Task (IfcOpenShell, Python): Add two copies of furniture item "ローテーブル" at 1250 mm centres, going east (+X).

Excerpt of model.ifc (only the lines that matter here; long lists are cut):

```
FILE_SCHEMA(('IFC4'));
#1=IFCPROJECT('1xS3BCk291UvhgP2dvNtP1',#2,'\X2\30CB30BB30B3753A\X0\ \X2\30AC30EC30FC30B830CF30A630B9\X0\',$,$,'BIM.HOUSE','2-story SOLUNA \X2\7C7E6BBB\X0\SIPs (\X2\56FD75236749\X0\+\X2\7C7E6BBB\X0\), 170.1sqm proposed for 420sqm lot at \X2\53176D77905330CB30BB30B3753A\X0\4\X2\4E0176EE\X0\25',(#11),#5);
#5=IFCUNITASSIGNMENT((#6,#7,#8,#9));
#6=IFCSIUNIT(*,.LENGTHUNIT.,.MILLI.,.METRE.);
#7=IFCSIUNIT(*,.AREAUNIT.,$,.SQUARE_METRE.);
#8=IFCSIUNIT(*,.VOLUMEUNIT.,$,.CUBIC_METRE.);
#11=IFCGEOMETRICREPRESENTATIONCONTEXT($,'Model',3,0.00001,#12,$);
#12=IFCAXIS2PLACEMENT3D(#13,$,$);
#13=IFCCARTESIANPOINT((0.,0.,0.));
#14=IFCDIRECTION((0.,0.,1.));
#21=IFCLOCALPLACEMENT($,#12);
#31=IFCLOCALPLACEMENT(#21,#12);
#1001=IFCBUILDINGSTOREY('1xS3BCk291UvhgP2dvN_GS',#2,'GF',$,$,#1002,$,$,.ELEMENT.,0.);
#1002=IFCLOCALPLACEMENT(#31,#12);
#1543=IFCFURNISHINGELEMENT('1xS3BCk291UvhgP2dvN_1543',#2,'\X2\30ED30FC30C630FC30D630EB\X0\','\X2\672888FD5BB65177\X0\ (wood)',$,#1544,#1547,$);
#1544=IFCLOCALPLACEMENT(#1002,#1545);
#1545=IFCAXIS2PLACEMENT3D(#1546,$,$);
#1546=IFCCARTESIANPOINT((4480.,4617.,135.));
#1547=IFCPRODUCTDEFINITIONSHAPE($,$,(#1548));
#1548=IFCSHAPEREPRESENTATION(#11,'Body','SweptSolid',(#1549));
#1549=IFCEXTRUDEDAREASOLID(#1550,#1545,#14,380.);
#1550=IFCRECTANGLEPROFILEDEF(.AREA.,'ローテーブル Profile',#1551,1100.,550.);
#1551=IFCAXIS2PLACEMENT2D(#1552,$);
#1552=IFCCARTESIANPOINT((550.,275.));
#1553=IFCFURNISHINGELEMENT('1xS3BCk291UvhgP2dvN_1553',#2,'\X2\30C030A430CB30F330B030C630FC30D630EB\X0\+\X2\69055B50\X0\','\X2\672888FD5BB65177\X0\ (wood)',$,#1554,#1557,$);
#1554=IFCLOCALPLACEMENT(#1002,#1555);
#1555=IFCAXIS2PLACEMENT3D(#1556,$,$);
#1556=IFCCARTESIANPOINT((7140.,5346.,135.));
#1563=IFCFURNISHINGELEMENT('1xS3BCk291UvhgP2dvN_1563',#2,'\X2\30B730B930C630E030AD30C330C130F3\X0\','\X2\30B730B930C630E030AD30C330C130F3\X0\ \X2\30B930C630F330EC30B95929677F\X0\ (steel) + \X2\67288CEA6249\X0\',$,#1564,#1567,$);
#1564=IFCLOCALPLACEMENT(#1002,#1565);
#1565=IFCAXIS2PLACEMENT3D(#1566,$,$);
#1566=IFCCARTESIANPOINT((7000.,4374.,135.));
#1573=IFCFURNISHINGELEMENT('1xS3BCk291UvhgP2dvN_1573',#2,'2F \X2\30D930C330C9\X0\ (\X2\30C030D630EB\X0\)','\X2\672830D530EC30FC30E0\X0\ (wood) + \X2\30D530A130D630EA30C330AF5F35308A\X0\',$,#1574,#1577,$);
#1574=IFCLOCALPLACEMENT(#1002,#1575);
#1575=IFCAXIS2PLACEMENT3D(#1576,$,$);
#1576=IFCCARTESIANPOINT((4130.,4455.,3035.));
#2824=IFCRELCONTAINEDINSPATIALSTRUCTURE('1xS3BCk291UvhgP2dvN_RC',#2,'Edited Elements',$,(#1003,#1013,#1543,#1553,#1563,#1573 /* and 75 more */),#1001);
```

```python
import numpy as np
import ifcopenshell
import ifcopenshell.api.geometry
import ifcopenshell.api.root
import ifcopenshell.util.element
import ifcopenshell.util.placement
import ifcopenshell.util.unit

model = ifcopenshell.open("model.ifc")
unit_scale = ifcopenshell.util.unit.calculate_unit_scale(model)


def reuse_history(source, copy):
    """copy_class also copies each property set's owner history, people and application; keep the originals."""
    for rel in copy.IsDefinedBy:
        if rel.is_a("IfcRelDefinesByProperties") and (history := rel.RelatingPropertyDefinition.OwnerHistory):
            rel.RelatingPropertyDefinition.OwnerHistory = source.OwnerHistory
            ifcopenshell.util.element.remove_deep2(model, history)


source = model.by_guid("1xS3BCk291UvhgP2dvN_1543")
base = ifcopenshell.util.placement.get_local_placement(source.ObjectPlacement)
step = np.array([1.0, 0.0, 0.0]) * 1.25 / unit_scale

for i in range(1, 3):
    copy = ifcopenshell.api.root.copy_class(model, product=source)
    copy.Representation = ifcopenshell.util.element.copy_deep(
        model, source.Representation, exclude=["IfcGeometricRepresentationContext", "IfcRepresentationMap"]
    )
    reuse_history(source, copy)
    matrix = base.copy()
    matrix[:3, 3] += i * step
    print("added at", matrix[:3, 3].round(3) + 0.0)
    ifcopenshell.api.geometry.edit_object_placement(model, product=copy, matrix=matrix, is_si=False)

model.write("model_edited.ifc")
```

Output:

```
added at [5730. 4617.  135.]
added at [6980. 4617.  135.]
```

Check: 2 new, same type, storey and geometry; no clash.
